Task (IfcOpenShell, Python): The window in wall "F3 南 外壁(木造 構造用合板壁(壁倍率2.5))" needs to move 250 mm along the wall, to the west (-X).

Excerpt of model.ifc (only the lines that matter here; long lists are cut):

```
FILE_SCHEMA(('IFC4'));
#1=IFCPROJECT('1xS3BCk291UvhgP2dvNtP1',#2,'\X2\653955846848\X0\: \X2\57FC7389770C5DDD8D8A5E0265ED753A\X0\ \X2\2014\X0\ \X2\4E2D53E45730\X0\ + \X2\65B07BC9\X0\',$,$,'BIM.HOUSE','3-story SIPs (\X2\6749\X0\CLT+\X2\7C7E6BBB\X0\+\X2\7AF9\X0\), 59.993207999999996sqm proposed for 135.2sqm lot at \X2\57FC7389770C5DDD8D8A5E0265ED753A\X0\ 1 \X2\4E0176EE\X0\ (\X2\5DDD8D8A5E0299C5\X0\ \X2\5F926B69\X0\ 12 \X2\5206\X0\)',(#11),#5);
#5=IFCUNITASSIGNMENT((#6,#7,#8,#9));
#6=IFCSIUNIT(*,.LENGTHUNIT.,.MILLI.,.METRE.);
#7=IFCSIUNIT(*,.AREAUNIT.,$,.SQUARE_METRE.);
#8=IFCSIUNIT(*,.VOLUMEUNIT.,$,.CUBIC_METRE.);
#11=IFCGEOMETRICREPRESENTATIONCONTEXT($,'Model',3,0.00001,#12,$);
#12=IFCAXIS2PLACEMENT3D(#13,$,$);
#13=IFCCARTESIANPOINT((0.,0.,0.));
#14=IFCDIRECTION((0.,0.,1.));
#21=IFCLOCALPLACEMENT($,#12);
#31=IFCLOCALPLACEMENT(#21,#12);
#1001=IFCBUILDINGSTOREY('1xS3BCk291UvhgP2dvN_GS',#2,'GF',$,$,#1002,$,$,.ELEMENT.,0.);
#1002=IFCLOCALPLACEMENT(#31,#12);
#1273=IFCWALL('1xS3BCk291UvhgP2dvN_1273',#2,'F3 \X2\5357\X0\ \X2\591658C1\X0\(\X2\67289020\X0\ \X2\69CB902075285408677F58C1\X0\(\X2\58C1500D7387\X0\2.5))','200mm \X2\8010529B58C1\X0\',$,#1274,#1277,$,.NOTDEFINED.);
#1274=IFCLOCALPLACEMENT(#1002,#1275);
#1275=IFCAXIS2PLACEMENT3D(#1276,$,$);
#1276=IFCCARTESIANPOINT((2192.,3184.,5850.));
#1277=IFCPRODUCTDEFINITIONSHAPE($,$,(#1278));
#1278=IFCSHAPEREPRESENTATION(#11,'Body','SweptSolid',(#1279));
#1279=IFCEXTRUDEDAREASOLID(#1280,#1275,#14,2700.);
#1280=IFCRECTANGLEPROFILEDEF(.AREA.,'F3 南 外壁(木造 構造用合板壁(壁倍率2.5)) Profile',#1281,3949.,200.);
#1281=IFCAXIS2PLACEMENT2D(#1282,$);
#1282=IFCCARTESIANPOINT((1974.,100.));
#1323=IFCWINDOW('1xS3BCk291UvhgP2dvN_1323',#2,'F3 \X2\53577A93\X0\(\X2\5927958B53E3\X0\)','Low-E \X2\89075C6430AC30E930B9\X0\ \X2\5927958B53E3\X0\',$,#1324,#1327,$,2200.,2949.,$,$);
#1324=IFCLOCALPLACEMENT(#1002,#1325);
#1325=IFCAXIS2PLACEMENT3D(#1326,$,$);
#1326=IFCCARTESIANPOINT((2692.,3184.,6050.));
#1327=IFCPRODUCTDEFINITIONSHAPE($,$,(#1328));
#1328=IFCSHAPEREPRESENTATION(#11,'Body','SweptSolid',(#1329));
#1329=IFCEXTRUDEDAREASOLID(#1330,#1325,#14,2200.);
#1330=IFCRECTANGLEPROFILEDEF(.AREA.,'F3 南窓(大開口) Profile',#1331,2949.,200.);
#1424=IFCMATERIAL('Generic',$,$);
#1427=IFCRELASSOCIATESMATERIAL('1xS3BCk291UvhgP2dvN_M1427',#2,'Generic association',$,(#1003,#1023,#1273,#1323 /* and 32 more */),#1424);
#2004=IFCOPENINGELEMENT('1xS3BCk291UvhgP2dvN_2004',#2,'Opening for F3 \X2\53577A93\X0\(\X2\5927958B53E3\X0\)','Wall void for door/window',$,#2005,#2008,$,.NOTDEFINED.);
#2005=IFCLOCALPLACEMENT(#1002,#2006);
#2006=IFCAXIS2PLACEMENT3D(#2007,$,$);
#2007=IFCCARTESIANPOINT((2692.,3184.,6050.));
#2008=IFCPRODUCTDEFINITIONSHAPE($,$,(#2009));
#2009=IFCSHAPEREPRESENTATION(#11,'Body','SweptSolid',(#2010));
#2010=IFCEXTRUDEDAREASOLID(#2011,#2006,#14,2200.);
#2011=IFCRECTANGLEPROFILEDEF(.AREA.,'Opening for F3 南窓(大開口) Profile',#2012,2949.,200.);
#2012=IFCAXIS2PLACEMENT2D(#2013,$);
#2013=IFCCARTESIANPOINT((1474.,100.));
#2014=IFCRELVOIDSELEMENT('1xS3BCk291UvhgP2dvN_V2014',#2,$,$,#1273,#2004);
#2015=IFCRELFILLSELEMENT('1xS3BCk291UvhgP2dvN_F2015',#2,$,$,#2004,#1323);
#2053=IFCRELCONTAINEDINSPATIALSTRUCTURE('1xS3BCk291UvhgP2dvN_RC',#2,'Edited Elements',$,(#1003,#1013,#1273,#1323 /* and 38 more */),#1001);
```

```python
import ifcopenshell
import ifcopenshell.api.geometry
import ifcopenshell.util.placement
import ifcopenshell.util.unit

model = ifcopenshell.open("model.ifc")
unit_scale = ifcopenshell.util.unit.calculate_unit_scale(model)

window = model.by_guid("1xS3BCk291UvhgP2dvN_1323")
opening = window.FillsVoids[0].RelatingOpeningElement
wall = opening.VoidsElements[0].RelatingBuildingElement

wall_matrix = ifcopenshell.util.placement.get_local_placement(wall.ObjectPlacement)
shift = wall_matrix[:3, 0] * -0.25 / unit_scale
before = ifcopenshell.util.placement.get_local_placement(window.ObjectPlacement)[:3, 3].copy()

# The window is not placed relative to its opening, so move both.
for product in (opening, window):
    matrix = ifcopenshell.util.placement.get_local_placement(product.ObjectPlacement)
    matrix[:3, 3] += shift
    ifcopenshell.api.geometry.edit_object_placement(model, product=product, matrix=matrix, is_si=False)

after = ifcopenshell.util.placement.get_local_placement(window.ObjectPlacement)[:3, 3]
print("window moved by", (after - before).round(3) + 0.0)

model.write("model_updated.ifc")
```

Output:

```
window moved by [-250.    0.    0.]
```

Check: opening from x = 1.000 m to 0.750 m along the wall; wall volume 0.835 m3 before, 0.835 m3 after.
